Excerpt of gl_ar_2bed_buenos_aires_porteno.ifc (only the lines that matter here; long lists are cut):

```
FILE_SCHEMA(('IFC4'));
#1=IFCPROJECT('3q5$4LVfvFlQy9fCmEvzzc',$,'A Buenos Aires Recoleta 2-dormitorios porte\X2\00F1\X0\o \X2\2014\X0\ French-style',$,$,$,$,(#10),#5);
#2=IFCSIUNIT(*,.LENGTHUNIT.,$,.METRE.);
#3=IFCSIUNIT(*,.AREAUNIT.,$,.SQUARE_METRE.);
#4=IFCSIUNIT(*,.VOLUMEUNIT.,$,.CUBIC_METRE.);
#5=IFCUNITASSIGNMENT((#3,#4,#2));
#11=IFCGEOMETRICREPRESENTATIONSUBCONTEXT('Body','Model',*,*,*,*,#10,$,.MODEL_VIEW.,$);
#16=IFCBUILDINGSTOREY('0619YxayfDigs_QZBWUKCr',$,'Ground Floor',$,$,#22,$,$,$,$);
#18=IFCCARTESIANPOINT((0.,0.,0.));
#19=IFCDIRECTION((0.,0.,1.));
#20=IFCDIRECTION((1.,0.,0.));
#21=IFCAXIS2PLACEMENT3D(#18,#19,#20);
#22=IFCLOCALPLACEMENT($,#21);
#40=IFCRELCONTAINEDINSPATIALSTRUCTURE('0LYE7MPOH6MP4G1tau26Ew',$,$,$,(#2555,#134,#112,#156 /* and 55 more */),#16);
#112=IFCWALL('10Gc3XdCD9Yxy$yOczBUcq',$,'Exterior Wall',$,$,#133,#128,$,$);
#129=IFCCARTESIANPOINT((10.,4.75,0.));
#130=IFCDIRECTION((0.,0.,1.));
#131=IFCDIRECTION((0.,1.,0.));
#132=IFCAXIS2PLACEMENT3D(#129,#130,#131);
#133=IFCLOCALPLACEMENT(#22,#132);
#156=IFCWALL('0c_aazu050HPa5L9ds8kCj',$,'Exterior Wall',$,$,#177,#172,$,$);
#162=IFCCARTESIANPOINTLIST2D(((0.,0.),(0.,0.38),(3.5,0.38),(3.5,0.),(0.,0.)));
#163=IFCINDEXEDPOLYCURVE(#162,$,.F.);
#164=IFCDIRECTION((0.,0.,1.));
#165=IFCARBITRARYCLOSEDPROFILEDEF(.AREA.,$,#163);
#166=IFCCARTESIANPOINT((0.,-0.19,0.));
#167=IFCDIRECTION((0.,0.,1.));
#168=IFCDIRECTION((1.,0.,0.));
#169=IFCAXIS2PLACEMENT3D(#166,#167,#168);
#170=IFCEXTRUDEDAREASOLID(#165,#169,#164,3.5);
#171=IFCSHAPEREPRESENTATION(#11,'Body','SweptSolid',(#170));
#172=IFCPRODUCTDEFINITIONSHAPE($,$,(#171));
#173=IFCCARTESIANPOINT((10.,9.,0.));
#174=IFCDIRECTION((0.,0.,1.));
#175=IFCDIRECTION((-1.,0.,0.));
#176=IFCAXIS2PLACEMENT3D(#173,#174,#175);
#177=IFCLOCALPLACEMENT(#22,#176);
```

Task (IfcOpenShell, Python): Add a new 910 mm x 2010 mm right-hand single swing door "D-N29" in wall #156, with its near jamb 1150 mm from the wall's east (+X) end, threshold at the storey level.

```python
import numpy as np
import ifcopenshell
import ifcopenshell.api.feature
import ifcopenshell.api.geometry
import ifcopenshell.api.root
import ifcopenshell.api.spatial
import ifcopenshell.geom
import ifcopenshell.util.element
import ifcopenshell.util.placement
import ifcopenshell.util.representation
import ifcopenshell.util.shape
import ifcopenshell.util.unit

model = ifcopenshell.open("gl_ar_2bed_buenos_aires_porteno.ifc")
unit_scale = ifcopenshell.util.unit.calculate_unit_scale(model)
settings = ifcopenshell.geom.settings()


def volume(element):
    """Net volume in cubic metres, openings subtracted."""
    shape = ifcopenshell.geom.create_shape(settings, element)
    return ifcopenshell.util.shape.get_volume(shape.geometry)


wall = model.by_guid("0c_aazu050HPa5L9ds8kCj")
storey = ifcopenshell.util.element.get_container(wall, ifc_class="IfcBuildingStorey")
context = ifcopenshell.util.representation.get_context(model, "Model", "Body", "MODEL_VIEW")
before = volume(wall)

width, height, from_end, sill = 0.91, 2.01, 1.15, 0.0  # metres

# The wall runs along its own X axis, and the end named is its -X end.
wall_shape = ifcopenshell.geom.create_shape(settings, wall)
x, y, z = ifcopenshell.util.shape.get_vertices(wall_shape.geometry).T
start = x.min() + from_end
face, thickness = float(y.min()), float(y.max() - y.min())
wall_matrix = ifcopenshell.util.placement.get_local_placement(wall.ObjectPlacement)
level = ifcopenshell.util.placement.get_local_placement(storey.ObjectPlacement)[2, 3]


def in_wall(x, y):
    """Placement at x, y metres in the wall's axes, at sill height."""
    matrix = wall_matrix.copy()
    matrix[:, 3] = wall_matrix @ np.array([x / unit_scale, y / unit_scale, 0.0, 1.0])
    matrix[2, 3] = level + sill / unit_scale
    return matrix


# Opening: a box that overshoots both wall faces by 50 mm.
opening = ifcopenshell.api.root.create_entity(model, ifc_class="IfcOpeningElement", predefined_type="OPENING")
box = ifcopenshell.api.geometry.add_wall_representation(
    model, context=context, length=width, height=height, thickness=thickness + 0.1
)
ifcopenshell.api.geometry.assign_representation(model, product=opening, representation=box)
ifcopenshell.api.geometry.edit_object_placement(model, product=opening, matrix=in_wall(start, face - 0.05), is_si=False)
ifcopenshell.api.feature.add_feature(model, feature=opening, element=wall)

door = ifcopenshell.api.root.create_entity(model, ifc_class="IfcDoor", name="D-N29", predefined_type="DOOR")
door.OverallWidth, door.OverallHeight = width / unit_scale, height / unit_scale
door.OperationType = "SINGLE_SWING_RIGHT"
body = ifcopenshell.api.geometry.add_door_representation(
    model,
    context=context,
    overall_width=door.OverallWidth,
    overall_height=door.OverallHeight,
    operation_type="SINGLE_SWING_RIGHT",
    lining_properties={"LiningDepth": thickness / unit_scale, "ThresholdDepth": thickness / unit_scale},
)
ifcopenshell.api.geometry.assign_representation(model, product=door, representation=body)
ifcopenshell.api.spatial.assign_container(model, products=[door], relating_structure=storey)
ifcopenshell.api.feature.add_filling(model, opening=opening, element=door)

# The lining spans the wall, so the door starts at the wall face.
ifcopenshell.api.geometry.edit_object_placement(model, product=door, matrix=in_wall(start, face), is_si=False)

after = volume(wall)

print(f"wall volume {before:.3f} -> {after:.3f} m3")

model.write("gl_ar_2bed_buenos_aires_porteno_updated.ifc")
```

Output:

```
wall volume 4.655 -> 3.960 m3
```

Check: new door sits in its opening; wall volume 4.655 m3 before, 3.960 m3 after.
